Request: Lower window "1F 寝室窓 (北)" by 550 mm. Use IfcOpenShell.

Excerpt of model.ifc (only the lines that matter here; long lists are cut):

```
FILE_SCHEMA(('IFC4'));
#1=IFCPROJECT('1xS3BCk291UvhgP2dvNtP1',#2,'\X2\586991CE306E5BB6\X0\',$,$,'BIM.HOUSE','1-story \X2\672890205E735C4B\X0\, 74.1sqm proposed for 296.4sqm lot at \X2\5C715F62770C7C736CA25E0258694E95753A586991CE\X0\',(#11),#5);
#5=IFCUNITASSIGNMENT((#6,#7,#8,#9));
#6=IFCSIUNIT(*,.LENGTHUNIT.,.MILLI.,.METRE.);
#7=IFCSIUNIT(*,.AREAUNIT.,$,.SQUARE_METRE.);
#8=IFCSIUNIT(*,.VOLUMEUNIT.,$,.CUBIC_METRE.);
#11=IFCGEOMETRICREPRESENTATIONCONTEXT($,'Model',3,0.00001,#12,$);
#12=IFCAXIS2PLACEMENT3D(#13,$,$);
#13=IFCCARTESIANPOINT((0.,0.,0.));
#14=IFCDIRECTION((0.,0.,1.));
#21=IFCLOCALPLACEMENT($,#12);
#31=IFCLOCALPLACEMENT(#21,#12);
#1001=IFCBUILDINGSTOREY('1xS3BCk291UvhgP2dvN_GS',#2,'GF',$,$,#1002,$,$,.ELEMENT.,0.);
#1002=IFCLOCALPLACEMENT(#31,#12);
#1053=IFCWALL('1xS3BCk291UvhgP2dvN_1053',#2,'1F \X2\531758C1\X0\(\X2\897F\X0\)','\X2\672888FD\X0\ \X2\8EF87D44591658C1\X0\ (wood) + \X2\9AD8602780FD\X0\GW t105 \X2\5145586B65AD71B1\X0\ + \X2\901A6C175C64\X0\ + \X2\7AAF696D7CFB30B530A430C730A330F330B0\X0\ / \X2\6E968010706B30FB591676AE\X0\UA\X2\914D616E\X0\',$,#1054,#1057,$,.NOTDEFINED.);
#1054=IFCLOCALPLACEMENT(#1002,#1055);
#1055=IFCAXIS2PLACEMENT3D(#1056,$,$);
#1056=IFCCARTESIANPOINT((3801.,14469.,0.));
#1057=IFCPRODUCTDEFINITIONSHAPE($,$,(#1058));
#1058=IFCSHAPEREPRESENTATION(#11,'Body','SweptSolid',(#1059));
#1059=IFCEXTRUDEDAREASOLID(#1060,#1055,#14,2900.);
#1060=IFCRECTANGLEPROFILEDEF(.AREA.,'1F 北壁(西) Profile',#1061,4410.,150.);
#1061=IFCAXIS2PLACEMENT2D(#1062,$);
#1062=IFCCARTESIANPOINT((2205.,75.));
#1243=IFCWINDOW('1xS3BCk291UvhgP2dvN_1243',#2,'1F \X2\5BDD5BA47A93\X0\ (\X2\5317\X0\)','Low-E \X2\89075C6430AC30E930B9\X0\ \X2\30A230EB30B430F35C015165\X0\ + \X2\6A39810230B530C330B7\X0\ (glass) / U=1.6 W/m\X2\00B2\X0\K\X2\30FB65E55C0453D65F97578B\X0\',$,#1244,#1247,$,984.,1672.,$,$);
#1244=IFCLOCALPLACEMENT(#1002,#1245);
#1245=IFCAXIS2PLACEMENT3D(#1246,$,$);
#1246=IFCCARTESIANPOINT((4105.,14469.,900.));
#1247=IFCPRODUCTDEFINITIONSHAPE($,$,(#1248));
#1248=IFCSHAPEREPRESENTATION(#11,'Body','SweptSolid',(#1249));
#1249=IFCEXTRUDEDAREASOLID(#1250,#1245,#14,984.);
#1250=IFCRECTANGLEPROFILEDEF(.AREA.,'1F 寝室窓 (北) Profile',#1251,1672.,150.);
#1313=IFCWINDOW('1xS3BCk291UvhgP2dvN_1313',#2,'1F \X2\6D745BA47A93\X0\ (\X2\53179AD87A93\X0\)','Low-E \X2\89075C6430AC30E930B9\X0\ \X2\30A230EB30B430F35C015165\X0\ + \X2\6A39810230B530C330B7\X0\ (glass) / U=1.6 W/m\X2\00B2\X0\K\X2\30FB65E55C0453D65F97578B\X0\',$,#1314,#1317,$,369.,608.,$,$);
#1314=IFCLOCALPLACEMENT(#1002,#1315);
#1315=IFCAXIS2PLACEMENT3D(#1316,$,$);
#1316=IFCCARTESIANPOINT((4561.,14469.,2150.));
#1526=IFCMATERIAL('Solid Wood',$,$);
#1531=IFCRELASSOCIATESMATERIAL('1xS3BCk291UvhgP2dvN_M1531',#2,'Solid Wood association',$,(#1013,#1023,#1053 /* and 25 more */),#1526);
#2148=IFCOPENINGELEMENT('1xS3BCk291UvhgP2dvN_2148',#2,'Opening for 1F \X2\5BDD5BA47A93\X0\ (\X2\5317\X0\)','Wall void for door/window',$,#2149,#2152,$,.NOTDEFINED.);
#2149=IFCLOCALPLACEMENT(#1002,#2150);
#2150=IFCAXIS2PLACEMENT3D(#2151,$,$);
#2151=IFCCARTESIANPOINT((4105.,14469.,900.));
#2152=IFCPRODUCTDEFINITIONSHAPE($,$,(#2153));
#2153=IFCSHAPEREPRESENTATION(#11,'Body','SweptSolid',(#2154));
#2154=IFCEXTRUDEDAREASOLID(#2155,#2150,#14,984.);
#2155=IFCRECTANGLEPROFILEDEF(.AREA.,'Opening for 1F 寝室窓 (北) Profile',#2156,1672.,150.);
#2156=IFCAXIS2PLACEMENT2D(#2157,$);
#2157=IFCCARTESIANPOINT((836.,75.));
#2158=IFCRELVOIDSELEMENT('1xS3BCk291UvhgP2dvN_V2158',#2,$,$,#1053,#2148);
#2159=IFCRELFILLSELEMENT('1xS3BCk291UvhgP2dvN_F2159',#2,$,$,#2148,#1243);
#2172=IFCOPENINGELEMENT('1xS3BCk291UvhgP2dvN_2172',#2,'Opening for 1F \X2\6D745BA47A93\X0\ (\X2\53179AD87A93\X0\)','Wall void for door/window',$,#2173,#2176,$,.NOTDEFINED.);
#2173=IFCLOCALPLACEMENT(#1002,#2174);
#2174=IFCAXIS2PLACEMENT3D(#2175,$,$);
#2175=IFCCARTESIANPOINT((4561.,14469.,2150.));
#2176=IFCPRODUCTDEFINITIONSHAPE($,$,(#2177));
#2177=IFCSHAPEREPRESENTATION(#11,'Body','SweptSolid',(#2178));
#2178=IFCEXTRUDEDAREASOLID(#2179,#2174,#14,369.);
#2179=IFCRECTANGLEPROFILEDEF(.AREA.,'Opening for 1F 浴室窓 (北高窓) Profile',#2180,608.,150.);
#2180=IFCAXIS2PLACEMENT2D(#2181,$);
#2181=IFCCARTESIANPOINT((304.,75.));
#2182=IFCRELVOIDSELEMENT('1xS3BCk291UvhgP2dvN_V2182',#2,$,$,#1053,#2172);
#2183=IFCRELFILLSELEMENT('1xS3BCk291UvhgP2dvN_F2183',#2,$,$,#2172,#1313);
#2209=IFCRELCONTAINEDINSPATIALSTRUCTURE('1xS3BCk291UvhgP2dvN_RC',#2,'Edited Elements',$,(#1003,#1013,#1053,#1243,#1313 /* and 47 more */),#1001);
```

```python
import numpy as np
import ifcopenshell
import ifcopenshell.api.geometry
import ifcopenshell.util.placement
import ifcopenshell.util.unit

model = ifcopenshell.open("model.ifc")
unit_scale = ifcopenshell.util.unit.calculate_unit_scale(model)

window = model.by_guid("1xS3BCk291UvhgP2dvN_1243")
opening = window.FillsVoids[0].RelatingOpeningElement
dz = -0.55 / unit_scale

shift = np.array([0.0, 0.0, dz])
# The window is not placed relative to its opening, so move both.
for product in (opening, window):
    matrix = ifcopenshell.util.placement.get_local_placement(product.ObjectPlacement)
    matrix[:3, 3] += shift
    ifcopenshell.api.geometry.edit_object_placement(model, product=product, matrix=matrix, is_si=False)

print(f"moved by {dz * unit_scale:+.3f} m")

model.write("model_updated.ifc")
```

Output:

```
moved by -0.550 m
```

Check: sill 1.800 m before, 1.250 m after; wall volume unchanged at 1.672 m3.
